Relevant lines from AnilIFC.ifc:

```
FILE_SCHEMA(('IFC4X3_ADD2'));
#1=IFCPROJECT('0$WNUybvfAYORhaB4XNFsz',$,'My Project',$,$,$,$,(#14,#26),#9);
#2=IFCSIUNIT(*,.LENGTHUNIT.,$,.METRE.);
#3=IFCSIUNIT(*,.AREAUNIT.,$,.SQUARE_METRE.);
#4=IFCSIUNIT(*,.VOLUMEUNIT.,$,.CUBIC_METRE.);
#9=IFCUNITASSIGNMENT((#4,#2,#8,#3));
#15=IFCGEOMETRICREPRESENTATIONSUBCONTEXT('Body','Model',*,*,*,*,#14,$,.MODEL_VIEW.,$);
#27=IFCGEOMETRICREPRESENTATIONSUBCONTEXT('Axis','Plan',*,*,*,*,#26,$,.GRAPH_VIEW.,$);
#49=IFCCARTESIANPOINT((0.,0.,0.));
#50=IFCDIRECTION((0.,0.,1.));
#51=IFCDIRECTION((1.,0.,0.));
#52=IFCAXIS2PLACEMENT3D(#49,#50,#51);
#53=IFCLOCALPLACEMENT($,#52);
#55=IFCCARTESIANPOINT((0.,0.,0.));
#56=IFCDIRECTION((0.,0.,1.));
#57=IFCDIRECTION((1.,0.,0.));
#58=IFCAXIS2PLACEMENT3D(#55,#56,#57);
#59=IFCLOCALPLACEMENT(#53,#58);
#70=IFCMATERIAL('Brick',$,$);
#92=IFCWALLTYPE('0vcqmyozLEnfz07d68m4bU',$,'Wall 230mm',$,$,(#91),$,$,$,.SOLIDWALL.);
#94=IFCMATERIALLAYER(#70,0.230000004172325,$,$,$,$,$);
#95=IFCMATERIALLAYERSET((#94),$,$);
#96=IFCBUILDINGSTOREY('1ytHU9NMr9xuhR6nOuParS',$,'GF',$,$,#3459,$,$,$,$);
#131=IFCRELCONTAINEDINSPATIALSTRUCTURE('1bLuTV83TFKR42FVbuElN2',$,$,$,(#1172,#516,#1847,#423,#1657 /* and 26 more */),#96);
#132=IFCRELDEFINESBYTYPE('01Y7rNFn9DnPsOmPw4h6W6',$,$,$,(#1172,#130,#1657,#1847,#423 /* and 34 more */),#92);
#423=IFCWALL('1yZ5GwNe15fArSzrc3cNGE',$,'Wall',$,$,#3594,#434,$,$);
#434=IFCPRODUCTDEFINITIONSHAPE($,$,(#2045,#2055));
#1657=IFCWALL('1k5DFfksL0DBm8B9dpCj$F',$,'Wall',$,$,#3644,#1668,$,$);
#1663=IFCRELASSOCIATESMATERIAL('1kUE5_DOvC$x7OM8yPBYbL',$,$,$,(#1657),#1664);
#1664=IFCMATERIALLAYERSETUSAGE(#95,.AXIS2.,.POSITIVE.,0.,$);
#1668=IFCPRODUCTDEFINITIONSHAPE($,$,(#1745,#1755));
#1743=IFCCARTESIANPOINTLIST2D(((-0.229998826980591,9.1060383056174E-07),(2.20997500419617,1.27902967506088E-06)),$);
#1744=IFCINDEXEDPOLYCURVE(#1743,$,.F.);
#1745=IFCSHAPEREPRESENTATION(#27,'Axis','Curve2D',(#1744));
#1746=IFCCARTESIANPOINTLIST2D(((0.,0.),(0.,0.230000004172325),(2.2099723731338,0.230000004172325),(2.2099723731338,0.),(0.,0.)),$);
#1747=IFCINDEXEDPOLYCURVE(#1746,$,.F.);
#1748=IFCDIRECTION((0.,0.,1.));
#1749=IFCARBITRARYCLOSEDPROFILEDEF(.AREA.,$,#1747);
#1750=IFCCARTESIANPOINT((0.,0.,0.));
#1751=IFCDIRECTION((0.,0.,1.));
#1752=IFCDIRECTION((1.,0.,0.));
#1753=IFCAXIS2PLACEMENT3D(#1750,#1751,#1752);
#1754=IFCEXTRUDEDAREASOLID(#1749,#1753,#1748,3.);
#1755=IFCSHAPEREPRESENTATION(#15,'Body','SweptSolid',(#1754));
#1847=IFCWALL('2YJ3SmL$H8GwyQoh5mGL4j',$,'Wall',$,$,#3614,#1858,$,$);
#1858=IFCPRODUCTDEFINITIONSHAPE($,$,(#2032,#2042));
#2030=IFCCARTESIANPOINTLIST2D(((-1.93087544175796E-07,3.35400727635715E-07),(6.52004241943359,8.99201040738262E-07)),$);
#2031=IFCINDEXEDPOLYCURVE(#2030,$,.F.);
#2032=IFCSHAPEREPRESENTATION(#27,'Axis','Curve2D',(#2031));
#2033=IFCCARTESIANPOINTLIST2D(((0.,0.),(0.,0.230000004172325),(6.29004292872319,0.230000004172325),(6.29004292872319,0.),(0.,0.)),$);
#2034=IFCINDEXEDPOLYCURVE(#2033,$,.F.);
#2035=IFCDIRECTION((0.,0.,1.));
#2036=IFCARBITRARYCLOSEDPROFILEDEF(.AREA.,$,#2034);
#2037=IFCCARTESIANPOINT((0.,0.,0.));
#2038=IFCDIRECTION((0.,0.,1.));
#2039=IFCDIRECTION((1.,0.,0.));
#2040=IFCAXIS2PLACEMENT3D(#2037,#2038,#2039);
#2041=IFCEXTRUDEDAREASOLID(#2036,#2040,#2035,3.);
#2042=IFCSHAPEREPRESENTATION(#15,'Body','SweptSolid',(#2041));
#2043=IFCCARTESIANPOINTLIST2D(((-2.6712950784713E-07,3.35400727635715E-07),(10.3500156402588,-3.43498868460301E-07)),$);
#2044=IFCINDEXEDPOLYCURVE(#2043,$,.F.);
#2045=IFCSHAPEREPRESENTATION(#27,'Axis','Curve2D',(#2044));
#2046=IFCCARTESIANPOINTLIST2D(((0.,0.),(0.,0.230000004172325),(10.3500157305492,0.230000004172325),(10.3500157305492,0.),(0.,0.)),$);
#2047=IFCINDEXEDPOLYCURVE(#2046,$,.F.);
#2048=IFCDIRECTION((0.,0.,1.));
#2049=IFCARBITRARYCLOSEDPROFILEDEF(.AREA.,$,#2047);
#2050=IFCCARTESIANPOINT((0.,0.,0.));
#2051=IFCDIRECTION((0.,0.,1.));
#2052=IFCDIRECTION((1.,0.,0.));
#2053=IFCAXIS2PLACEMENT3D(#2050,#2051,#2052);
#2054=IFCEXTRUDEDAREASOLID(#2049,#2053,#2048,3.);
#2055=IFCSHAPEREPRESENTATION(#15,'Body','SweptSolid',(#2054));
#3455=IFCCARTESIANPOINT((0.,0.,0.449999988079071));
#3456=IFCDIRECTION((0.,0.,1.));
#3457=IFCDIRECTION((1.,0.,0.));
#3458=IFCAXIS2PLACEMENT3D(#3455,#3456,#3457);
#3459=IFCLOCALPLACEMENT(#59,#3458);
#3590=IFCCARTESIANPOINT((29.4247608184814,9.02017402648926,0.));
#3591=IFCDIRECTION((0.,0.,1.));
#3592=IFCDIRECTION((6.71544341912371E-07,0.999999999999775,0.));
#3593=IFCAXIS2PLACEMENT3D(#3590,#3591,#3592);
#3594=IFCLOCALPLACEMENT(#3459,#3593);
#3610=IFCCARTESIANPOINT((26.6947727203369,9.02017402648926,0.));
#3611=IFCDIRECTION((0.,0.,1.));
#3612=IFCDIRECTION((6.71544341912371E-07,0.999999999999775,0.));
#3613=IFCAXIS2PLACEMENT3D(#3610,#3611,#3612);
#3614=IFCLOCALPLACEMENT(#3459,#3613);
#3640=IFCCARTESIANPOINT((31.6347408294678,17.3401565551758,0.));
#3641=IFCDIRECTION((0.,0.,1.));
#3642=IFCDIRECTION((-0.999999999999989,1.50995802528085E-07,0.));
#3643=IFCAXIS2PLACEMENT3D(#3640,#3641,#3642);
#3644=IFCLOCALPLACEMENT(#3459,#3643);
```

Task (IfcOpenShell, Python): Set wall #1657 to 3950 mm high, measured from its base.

```python
import ifcopenshell
import ifcopenshell.geom
import ifcopenshell.util.representation
import ifcopenshell.util.shape
import ifcopenshell.util.unit

model = ifcopenshell.open("AnilIFC.ifc")
unit_scale = ifcopenshell.util.unit.calculate_unit_scale(model)
settings = ifcopenshell.geom.settings()


def volume(element):
    """Net volume in cubic metres, openings subtracted."""
    shape = ifcopenshell.geom.create_shape(settings, element)
    return ifcopenshell.util.shape.get_volume(shape.geometry)


wall = model.by_guid("1k5DFfksL0DBm8B9dpCj$F")
before = volume(wall)

body = ifcopenshell.util.representation.get_representation(wall, "Model", "Body")
solid = body.Items[0]
old_height = solid.Depth
solid.Depth = 3.95 / unit_scale
after = volume(wall)

print(f"height {old_height:g} -> {solid.Depth:g}, volume {before:.3f} -> {after:.3f} m3")

model.write("AnilIFC-out.ifc")
```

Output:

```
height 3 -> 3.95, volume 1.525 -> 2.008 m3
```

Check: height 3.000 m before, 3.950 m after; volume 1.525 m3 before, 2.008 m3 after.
